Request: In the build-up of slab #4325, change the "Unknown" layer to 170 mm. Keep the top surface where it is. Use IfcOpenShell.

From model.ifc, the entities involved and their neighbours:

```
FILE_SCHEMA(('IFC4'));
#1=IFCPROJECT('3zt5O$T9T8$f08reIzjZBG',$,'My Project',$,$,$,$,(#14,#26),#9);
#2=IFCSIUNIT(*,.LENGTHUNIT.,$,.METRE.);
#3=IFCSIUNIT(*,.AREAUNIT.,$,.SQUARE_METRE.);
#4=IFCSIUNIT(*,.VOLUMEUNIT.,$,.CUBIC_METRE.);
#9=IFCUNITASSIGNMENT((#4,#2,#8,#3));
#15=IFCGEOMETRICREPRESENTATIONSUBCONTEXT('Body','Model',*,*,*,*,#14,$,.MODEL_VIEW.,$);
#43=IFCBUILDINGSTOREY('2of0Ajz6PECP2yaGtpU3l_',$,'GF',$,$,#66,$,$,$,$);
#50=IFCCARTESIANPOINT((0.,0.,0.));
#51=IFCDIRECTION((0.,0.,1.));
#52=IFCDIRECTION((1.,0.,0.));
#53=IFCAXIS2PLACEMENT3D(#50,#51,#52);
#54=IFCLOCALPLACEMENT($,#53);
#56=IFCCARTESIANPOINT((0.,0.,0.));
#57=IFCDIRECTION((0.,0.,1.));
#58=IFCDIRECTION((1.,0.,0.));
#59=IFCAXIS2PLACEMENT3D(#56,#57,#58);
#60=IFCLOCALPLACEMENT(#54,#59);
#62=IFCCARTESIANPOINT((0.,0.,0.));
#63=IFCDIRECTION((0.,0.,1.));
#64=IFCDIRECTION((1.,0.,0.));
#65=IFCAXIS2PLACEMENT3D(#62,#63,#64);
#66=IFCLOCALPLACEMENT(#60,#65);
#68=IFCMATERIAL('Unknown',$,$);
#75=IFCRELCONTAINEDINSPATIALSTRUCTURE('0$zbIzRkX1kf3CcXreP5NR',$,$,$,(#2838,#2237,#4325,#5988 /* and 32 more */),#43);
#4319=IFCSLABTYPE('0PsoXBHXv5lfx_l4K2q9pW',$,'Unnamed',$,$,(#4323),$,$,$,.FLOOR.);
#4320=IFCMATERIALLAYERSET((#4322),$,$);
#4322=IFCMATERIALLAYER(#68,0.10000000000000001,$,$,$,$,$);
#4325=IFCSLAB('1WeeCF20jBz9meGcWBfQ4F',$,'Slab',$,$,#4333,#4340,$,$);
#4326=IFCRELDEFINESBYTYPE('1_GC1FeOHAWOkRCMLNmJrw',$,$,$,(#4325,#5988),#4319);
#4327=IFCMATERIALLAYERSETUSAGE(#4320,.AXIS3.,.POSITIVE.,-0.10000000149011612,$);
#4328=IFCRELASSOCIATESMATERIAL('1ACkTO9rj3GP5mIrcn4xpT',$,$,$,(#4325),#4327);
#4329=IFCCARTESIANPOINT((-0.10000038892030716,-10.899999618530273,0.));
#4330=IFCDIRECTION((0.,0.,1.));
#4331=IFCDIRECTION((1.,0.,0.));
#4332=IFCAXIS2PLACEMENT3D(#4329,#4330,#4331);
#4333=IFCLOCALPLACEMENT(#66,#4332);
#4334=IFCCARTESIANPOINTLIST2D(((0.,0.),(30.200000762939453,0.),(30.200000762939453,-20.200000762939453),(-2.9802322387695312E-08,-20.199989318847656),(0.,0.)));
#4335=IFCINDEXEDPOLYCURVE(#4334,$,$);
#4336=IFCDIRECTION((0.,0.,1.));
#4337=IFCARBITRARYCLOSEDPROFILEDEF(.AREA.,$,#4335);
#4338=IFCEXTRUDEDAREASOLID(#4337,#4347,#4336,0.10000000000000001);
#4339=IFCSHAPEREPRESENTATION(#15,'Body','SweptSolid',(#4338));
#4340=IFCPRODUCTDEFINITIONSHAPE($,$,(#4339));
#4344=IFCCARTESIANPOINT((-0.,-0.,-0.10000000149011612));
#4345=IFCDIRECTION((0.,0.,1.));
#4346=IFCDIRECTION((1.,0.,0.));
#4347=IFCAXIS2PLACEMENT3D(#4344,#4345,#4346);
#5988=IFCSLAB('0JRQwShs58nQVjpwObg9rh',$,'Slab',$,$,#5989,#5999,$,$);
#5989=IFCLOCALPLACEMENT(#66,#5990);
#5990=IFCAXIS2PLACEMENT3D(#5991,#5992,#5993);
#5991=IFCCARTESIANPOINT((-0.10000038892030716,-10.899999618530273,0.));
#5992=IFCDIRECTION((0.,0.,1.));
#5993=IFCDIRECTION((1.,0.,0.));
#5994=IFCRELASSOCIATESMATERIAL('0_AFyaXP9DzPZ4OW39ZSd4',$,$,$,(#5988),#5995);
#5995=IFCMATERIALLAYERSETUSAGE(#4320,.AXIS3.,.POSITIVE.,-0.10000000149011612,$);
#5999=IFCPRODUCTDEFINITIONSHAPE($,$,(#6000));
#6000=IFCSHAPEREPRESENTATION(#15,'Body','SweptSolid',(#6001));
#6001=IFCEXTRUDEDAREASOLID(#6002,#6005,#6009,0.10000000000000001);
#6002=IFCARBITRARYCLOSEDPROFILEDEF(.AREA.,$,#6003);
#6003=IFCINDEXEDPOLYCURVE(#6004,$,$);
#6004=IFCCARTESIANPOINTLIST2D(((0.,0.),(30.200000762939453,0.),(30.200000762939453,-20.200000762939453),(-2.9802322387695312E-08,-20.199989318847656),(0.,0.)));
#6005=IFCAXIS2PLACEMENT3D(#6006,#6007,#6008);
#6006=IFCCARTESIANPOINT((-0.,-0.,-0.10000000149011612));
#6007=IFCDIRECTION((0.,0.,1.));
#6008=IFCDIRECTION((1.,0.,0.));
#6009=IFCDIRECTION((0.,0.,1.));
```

```python
import ifcopenshell
import ifcopenshell.util.element
import ifcopenshell.util.representation

model = ifcopenshell.open("model.ifc")

layer_set = model.by_id(4320)
layer = next(l for l in layer_set.MaterialLayers if l.Material and l.Material.Name == "Unknown")
change = 0.17 - layer.LayerThickness
layer.LayerThickness += change

# The layer set is shared, so every slab that uses it gets the new thickness.
slabs = [e for e in ifcopenshell.util.element.get_elements_by_material(model, layer_set) if e.is_a("IfcSlab")]
for slab in sorted(slabs, key=lambda e: e.id()):
    body = ifcopenshell.util.representation.get_representation(slab, "Model", "Body")
    solid = body.Items[0]
    old_depth = solid.Depth
    solid.Depth += change
    # Extruded upwards: lower the start of the extrusion so the top stays.
    x, y, z = solid.Position.Location.Coordinates
    solid.Position.Location = model.createIfcCartesianPoint((x, y, z - change))
    print(slab.id(), f"{old_depth:g} -> {solid.Depth:g}")

# The layers are counted up from the underside, which has moved.
for usage in {ifcopenshell.util.element.get_material(slab) for slab in slabs}:
    usage.OffsetFromReferenceLine -= change

model.write("model-out.ifc")
```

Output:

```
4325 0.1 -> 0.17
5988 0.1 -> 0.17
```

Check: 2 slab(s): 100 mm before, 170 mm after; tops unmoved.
